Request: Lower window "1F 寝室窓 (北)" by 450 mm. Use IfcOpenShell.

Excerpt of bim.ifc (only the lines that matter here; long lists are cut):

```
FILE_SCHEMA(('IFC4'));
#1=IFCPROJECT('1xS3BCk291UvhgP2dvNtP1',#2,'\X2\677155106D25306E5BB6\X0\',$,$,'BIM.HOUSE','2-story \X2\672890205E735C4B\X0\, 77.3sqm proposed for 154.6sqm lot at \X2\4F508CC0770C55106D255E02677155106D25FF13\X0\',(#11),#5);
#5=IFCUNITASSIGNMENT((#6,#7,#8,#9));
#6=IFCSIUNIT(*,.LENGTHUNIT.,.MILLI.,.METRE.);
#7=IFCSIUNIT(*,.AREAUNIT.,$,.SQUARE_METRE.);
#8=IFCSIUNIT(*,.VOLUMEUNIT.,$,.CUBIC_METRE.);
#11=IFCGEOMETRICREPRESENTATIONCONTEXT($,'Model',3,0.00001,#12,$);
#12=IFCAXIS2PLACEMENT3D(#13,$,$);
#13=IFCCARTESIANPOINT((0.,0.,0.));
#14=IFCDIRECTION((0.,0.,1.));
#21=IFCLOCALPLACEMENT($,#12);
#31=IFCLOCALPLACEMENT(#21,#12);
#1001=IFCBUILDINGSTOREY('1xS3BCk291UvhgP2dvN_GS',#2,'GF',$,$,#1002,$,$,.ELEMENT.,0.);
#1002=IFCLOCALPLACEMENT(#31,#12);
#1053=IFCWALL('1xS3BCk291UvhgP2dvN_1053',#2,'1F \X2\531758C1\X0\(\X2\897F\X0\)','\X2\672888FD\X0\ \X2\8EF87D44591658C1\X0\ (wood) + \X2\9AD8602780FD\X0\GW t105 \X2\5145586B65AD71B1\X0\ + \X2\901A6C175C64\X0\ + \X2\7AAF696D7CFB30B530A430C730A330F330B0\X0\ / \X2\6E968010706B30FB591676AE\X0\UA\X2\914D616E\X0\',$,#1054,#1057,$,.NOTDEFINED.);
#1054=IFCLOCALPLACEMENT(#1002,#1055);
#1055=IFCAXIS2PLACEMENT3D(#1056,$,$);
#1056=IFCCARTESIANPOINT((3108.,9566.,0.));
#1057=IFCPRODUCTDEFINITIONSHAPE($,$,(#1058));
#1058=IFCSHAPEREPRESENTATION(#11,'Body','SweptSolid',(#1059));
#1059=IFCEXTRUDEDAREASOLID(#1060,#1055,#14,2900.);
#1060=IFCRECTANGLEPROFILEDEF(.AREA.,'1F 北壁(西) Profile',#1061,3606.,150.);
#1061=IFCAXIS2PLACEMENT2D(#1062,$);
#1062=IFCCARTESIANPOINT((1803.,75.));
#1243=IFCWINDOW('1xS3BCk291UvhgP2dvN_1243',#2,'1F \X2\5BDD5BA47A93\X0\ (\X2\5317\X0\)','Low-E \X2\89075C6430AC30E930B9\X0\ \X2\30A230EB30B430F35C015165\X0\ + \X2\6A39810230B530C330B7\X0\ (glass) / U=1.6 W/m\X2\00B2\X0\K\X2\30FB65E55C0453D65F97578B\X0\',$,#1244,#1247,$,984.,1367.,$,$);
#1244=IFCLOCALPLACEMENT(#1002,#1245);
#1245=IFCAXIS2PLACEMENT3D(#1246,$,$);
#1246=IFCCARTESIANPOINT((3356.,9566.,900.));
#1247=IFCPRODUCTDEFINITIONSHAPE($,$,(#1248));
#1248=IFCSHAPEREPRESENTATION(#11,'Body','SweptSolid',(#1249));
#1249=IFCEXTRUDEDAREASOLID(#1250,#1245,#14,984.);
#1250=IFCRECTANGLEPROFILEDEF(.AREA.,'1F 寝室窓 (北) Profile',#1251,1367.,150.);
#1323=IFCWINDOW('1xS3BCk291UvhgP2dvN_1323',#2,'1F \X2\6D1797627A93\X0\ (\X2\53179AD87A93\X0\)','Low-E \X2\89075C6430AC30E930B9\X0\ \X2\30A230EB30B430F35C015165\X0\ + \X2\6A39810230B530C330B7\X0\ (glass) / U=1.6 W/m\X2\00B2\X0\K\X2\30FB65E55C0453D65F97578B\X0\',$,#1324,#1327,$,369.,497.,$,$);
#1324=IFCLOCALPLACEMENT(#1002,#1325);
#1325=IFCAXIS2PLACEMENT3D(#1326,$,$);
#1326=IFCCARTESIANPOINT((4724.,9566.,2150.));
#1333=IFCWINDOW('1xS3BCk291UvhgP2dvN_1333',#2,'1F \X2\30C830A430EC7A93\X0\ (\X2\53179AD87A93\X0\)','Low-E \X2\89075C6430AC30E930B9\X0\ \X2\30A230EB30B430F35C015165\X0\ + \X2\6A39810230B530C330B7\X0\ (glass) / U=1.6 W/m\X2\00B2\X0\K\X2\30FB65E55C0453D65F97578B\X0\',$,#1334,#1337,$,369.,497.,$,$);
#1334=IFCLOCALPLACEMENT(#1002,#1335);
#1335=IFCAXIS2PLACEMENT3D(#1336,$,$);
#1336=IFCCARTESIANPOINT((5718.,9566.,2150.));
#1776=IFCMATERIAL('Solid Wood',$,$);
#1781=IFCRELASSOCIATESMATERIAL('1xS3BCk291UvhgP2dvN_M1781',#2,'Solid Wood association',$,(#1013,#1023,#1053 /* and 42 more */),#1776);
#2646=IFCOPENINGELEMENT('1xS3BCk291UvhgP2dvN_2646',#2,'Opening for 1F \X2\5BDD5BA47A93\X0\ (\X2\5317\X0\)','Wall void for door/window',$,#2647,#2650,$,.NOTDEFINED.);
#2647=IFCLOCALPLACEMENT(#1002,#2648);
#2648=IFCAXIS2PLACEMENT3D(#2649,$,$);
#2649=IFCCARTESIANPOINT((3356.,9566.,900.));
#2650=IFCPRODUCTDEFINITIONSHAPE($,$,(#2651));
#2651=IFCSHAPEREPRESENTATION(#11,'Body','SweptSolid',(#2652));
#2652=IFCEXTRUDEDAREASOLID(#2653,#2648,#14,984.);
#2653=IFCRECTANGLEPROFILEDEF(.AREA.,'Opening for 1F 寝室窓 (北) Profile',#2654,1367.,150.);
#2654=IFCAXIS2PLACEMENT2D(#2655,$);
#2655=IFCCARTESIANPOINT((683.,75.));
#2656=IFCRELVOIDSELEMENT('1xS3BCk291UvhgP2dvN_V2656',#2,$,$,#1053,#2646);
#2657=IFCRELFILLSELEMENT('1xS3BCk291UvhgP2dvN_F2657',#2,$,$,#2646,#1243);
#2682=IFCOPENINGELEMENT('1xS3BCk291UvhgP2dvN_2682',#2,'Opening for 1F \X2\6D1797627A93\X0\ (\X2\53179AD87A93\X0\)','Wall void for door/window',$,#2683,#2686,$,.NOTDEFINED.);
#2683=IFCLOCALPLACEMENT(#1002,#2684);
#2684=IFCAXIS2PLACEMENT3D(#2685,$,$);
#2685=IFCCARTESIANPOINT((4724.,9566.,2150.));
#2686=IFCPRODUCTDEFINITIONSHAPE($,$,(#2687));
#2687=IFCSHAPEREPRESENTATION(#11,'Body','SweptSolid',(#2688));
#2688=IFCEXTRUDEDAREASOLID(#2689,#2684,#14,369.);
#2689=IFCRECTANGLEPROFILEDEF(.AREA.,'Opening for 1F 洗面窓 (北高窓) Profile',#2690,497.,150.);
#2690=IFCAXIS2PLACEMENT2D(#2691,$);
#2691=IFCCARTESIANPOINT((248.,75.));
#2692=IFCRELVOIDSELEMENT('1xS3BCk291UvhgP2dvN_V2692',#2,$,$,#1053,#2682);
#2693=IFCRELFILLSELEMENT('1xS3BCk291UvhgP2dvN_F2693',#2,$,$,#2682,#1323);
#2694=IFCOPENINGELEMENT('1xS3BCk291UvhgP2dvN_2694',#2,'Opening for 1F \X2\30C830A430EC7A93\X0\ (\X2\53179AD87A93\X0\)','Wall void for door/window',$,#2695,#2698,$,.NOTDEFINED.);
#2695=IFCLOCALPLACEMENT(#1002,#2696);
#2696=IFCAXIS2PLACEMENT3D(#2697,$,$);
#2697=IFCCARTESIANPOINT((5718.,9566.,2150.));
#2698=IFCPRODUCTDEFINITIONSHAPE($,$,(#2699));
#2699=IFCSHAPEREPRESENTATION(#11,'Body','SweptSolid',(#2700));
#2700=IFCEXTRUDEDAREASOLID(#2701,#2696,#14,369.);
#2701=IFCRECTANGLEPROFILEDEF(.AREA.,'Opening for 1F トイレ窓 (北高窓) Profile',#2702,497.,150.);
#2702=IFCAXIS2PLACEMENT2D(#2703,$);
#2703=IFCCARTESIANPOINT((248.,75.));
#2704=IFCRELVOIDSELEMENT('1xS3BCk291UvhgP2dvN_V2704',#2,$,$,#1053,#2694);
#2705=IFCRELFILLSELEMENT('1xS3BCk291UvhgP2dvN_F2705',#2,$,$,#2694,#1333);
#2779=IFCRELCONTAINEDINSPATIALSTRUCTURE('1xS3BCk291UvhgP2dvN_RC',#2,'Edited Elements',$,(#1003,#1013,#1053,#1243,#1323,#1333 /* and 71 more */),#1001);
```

```python
import numpy as np
import ifcopenshell
import ifcopenshell.api.geometry
import ifcopenshell.util.placement
import ifcopenshell.util.unit

model = ifcopenshell.open("bim.ifc")
unit_scale = ifcopenshell.util.unit.calculate_unit_scale(model)

window = model.by_id(1243)
opening = window.FillsVoids[0].RelatingOpeningElement
dz = -0.45 / unit_scale

shift = np.array([0.0, 0.0, dz])
# The window is not placed relative to its opening, so move both.
for product in (opening, window):
    matrix = ifcopenshell.util.placement.get_local_placement(product.ObjectPlacement)
    matrix[:3, 3] += shift
    ifcopenshell.api.geometry.edit_object_placement(model, product=product, matrix=matrix, is_si=False)

print(f"moved by {dz * unit_scale:+.3f} m")

model.write("bim_edited.ifc")
```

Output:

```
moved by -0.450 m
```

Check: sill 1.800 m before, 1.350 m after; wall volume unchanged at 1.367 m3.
